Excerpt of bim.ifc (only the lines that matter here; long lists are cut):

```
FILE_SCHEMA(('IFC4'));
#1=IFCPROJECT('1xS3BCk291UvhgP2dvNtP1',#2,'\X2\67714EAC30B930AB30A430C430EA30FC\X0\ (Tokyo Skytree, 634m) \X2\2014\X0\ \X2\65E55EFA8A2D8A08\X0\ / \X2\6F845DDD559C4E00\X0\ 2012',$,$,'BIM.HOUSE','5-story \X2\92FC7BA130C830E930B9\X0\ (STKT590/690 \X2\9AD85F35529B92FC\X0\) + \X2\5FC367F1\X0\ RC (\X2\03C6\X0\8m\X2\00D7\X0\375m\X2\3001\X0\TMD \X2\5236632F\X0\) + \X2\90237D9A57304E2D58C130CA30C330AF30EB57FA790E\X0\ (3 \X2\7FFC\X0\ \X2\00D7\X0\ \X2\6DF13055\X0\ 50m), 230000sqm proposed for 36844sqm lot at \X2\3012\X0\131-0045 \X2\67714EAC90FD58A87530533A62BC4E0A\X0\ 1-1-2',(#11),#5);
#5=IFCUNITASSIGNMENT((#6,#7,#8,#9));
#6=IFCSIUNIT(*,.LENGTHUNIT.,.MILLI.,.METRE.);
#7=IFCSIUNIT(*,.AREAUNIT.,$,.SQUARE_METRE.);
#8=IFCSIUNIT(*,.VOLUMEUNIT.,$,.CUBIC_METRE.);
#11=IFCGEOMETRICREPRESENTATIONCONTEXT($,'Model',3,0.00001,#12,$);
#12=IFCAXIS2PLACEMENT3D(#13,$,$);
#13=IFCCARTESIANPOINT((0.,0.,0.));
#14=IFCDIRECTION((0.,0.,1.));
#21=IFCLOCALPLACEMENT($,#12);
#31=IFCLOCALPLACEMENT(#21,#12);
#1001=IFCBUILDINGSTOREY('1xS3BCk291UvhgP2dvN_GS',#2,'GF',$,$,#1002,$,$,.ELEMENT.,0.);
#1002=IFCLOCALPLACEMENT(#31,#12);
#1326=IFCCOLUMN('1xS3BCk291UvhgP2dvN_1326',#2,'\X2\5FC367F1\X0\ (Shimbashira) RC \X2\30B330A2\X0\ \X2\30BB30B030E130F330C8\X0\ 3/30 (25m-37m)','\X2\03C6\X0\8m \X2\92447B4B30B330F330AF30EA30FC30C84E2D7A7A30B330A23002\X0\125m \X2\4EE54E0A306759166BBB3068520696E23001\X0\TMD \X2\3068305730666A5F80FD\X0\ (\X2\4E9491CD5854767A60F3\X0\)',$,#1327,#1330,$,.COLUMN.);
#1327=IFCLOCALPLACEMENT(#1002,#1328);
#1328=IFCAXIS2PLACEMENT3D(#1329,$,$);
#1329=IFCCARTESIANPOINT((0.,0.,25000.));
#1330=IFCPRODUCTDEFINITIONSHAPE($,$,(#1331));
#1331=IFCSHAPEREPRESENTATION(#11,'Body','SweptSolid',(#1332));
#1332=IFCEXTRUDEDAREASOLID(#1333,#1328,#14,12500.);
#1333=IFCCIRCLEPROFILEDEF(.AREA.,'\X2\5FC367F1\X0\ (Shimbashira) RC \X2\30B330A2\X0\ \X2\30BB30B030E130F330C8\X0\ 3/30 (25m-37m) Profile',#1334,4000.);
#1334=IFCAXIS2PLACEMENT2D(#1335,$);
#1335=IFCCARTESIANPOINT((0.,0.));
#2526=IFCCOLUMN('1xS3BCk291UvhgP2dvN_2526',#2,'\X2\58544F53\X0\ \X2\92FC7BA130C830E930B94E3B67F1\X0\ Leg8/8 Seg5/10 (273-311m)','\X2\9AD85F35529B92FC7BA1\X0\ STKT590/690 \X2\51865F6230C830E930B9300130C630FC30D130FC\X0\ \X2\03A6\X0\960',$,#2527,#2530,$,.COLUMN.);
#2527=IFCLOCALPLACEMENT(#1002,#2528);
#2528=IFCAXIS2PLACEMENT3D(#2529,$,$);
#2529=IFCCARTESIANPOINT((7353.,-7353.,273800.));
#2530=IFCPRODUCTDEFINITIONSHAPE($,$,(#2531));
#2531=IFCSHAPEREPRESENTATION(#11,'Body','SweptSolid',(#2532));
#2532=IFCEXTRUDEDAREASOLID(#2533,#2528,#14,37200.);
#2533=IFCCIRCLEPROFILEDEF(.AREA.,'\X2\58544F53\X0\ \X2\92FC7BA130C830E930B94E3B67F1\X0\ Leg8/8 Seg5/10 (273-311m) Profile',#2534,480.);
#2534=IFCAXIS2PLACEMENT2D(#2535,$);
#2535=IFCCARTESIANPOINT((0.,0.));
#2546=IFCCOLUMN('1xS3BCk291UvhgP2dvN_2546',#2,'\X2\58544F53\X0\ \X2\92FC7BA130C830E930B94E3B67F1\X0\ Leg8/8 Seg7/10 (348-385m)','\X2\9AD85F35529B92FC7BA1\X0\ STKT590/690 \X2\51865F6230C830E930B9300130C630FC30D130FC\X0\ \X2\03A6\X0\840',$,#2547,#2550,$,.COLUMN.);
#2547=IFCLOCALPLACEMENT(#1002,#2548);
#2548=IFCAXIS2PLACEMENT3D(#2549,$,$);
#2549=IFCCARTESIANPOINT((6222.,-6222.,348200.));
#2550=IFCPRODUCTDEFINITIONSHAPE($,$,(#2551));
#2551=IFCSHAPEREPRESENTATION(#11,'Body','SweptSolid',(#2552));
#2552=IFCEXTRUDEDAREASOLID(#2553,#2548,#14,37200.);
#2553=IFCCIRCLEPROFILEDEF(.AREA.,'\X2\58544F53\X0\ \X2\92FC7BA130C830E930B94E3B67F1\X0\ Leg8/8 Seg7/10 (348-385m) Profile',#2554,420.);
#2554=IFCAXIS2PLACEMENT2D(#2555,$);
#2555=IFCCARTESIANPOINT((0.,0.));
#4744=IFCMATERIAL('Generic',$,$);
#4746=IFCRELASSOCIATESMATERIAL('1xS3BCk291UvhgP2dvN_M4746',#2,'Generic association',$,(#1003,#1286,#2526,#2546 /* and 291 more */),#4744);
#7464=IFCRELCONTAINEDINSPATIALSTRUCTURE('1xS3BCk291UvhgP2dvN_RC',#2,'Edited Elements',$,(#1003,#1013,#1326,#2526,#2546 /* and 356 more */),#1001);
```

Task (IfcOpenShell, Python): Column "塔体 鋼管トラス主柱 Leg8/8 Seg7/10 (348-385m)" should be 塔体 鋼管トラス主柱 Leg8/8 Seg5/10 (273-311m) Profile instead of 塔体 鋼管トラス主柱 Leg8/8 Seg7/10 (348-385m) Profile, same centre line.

```python
import ifcopenshell
import ifcopenshell.util.element

model = ifcopenshell.open("bim.ifc")

member = model.by_id(2546)
source = next(p for p in model.by_type("IfcCircleProfileDef") if p.ProfileName == "塔体 鋼管トラス主柱 Leg8/8 Seg5/10 (273-311m) Profile")

body = next(r for r in member.Representation.Representations if r.RepresentationIdentifier == "Body")
solid = body.Items[0]
old_profile = solid.SweptArea

# Copy the section's sizes but keep this member's own profile position.
profile = ifcopenshell.util.element.copy(model, source)
profile.Position = old_profile.Position
solid.SweptArea = profile
if not model.get_total_inverses(old_profile):
    ifcopenshell.util.element.remove_deep2(model, old_profile)

print(solid.SweptArea)

model.write("bim_rev.ifc")
```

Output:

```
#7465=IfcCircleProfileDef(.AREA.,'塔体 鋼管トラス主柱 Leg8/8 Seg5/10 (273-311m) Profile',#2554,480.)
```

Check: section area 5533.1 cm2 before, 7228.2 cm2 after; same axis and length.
